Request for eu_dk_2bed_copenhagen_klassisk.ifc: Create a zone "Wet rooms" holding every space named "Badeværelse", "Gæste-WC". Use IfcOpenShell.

First a look at what the model holds.

```python
import ifcopenshell

model = ifcopenshell.open("eu_dk_2bed_copenhagen_klassisk.ifc")
print(model.schema)
seen = {}
for space in model.by_type("IfcSpace"):
    seen[space.LongName] = seen.get(space.LongName, 0) + 1
for name, count in sorted(seen.items(), key=str):
    print(count, "x", name)
print("zones:", [z.Name for z in model.by_type("IfcZone")][:20])
```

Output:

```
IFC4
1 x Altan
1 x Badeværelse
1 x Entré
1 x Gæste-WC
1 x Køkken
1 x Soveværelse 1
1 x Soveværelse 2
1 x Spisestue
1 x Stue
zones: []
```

```python
import ifcopenshell
import ifcopenshell.api.group
import ifcopenshell.api.root

model = ifcopenshell.open("eu_dk_2bed_copenhagen_klassisk.ifc")

names = {"Badeværelse", "Gæste-WC"}
spaces = [s for s in model.by_type("IfcSpace") if s.LongName in names]

zone = ifcopenshell.api.root.create_entity(model, ifc_class="IfcZone", name="Wet rooms")
ifcopenshell.api.group.assign_group(model, products=spaces, group=zone)
print(len(spaces), "spaces in", zone.Name)

model.write("eu_dk_2bed_copenhagen_klassisk_v2.ifc")
```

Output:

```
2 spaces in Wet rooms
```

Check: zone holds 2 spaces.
